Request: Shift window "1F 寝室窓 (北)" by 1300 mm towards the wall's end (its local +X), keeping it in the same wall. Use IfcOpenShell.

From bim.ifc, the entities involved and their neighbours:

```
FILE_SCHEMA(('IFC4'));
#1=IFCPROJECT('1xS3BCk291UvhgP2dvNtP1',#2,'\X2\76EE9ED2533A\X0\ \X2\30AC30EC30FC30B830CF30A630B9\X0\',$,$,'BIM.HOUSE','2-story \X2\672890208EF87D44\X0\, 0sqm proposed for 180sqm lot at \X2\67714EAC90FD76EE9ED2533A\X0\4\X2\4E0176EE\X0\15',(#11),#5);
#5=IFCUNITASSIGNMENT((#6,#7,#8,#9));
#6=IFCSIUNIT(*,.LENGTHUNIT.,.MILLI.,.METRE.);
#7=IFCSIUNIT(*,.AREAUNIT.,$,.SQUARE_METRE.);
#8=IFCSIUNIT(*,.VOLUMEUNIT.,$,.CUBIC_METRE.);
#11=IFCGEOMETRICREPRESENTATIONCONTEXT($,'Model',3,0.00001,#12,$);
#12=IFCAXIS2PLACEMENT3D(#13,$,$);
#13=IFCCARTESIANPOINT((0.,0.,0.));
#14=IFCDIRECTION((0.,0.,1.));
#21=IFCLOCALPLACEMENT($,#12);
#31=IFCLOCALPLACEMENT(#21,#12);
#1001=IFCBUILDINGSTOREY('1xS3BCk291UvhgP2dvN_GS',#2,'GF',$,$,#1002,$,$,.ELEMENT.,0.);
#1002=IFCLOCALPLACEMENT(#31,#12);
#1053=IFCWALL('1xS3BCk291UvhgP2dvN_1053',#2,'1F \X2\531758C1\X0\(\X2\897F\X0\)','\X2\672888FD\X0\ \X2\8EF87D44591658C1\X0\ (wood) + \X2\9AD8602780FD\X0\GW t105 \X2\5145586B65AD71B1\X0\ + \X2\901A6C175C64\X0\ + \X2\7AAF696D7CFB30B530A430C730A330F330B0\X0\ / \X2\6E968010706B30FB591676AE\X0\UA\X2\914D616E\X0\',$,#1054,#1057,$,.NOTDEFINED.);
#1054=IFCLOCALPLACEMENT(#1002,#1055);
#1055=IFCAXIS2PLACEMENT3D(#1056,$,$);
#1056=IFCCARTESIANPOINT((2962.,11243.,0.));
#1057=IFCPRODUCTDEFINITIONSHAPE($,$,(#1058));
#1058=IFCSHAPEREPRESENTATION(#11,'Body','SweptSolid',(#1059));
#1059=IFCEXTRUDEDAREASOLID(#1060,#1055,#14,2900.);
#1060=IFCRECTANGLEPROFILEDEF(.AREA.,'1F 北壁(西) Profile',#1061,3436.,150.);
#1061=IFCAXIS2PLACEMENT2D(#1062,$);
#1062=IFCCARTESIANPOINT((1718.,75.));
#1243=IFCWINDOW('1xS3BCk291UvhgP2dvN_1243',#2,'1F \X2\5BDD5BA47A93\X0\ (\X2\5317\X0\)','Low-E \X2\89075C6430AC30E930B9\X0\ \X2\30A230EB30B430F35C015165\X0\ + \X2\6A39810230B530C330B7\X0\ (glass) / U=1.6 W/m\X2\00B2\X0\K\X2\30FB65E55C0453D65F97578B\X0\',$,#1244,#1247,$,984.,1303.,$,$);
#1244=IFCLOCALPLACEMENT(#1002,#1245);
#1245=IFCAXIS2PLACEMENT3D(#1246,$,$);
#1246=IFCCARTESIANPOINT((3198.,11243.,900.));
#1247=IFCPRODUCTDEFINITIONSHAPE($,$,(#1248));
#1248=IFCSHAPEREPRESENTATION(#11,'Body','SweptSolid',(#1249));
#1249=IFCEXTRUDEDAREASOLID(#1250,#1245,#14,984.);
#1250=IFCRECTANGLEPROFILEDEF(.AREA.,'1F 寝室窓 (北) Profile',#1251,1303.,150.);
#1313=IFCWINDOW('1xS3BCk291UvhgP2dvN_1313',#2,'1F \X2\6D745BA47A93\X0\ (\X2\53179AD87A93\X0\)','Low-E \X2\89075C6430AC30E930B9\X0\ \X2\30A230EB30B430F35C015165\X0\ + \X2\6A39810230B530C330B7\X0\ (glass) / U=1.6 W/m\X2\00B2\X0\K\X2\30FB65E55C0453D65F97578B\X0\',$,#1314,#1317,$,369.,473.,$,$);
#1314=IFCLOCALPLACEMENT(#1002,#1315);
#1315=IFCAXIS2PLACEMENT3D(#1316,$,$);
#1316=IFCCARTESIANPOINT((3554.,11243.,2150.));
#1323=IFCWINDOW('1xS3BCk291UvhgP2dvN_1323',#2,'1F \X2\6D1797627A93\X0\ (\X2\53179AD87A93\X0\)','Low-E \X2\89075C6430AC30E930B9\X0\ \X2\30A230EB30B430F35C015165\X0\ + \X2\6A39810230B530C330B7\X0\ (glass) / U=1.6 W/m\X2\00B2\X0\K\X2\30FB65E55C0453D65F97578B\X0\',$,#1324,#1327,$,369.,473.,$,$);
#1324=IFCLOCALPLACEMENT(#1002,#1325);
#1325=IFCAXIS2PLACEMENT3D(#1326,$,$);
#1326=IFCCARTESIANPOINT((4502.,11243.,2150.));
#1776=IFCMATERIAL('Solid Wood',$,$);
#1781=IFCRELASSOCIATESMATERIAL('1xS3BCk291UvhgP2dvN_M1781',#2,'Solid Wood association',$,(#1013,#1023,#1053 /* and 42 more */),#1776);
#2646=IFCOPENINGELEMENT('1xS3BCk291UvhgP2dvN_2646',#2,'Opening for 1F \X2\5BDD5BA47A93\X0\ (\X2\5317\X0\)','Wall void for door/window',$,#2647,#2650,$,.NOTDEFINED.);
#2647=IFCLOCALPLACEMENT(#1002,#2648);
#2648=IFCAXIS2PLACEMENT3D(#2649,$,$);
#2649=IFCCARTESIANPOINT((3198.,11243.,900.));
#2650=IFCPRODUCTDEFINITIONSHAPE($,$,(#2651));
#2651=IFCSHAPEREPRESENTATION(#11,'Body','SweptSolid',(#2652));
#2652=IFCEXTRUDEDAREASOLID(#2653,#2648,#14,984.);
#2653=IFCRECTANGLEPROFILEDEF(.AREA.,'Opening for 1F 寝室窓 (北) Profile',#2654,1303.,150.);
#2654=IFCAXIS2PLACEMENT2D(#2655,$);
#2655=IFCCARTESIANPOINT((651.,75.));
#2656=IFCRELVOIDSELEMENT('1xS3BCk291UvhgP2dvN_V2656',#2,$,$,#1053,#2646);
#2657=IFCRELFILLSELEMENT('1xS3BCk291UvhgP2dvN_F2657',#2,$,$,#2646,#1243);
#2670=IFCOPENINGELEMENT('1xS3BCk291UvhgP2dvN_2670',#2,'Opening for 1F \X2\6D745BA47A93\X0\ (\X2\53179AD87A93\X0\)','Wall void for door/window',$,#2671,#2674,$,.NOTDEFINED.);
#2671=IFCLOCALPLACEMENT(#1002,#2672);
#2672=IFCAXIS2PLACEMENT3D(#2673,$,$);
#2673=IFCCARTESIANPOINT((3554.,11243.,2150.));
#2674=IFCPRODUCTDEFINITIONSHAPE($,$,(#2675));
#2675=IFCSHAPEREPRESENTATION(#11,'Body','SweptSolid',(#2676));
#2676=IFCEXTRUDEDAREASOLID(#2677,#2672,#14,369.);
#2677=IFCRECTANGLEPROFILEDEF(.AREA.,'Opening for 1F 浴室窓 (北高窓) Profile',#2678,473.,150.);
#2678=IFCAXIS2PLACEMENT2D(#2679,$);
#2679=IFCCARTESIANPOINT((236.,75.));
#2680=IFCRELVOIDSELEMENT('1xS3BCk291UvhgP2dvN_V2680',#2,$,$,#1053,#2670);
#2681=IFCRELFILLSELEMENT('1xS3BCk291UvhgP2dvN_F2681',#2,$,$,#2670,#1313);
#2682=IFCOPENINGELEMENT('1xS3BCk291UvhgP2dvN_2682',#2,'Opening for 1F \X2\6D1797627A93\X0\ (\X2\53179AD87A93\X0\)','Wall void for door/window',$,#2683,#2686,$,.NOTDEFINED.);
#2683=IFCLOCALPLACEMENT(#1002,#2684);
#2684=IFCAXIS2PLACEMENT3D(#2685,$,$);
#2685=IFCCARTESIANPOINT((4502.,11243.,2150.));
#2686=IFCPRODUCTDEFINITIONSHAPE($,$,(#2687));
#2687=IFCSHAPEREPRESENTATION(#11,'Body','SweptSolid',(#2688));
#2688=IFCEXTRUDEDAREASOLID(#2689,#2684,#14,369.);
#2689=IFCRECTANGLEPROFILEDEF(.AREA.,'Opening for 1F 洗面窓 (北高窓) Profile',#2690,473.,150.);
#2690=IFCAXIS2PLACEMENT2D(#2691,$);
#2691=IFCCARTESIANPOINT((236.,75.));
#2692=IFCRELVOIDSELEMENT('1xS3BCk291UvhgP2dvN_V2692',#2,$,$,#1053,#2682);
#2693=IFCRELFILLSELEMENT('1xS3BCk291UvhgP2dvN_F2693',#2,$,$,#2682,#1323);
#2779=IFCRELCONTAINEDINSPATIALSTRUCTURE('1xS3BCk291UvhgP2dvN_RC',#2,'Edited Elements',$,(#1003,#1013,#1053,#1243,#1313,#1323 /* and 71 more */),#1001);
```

```python
import ifcopenshell
import ifcopenshell.api.geometry
import ifcopenshell.util.placement

model = ifcopenshell.open("bim.ifc")

window = model.by_guid("1xS3BCk291UvhgP2dvN_1243")
opening = window.FillsVoids[0].RelatingOpeningElement
wall = opening.VoidsElements[0].RelatingBuildingElement

wall_matrix = ifcopenshell.util.placement.get_local_placement(wall.ObjectPlacement)
shift = wall_matrix[:3, 0] * 1300.0
before = ifcopenshell.util.placement.get_local_placement(window.ObjectPlacement)[:3, 3].copy()

# The window is not placed relative to its opening, so move both.
for product in (opening, window):
    matrix = ifcopenshell.util.placement.get_local_placement(product.ObjectPlacement)
    matrix[:3, 3] += shift
    ifcopenshell.api.geometry.edit_object_placement(model, product=product, matrix=matrix, is_si=False)

after = ifcopenshell.util.placement.get_local_placement(window.ObjectPlacement)[:3, 3]
print("window moved by", (after - before).round(3) + 0.0)

model.write("bim_rev.ifc")
```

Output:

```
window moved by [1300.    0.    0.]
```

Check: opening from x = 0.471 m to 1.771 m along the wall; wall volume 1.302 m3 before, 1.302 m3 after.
